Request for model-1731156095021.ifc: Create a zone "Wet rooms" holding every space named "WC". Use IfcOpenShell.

First a look at what the model holds.

```python
import ifcopenshell

model = ifcopenshell.open("model-1731156095021.ifc")
print(model.schema)
seen = {}
for space in model.by_type("IfcSpace"):
    seen[space.LongName] = seen.get(space.LongName, 0) + 1
for name, count in sorted(seen.items(), key=str):
    print(count, "x", name)
print("zones:", [z.Name for z in model.by_type("IfcZone")][:20])
```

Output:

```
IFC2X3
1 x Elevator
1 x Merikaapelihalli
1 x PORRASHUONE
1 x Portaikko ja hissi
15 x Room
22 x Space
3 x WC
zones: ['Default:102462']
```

```python
import ifcopenshell
import ifcopenshell.api.group
import ifcopenshell.api.root

model = ifcopenshell.open("model-1731156095021.ifc")

names = {"WC"}
spaces = [s for s in model.by_type("IfcSpace") if s.LongName in names]

zone = ifcopenshell.api.root.create_entity(model, ifc_class="IfcZone", name="Wet rooms")
ifcopenshell.api.group.assign_group(model, products=spaces, group=zone)
print(len(spaces), "spaces in", zone.Name)

model.write("model-1731156095021_updated.ifc")
```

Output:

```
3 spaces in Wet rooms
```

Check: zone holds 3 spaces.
